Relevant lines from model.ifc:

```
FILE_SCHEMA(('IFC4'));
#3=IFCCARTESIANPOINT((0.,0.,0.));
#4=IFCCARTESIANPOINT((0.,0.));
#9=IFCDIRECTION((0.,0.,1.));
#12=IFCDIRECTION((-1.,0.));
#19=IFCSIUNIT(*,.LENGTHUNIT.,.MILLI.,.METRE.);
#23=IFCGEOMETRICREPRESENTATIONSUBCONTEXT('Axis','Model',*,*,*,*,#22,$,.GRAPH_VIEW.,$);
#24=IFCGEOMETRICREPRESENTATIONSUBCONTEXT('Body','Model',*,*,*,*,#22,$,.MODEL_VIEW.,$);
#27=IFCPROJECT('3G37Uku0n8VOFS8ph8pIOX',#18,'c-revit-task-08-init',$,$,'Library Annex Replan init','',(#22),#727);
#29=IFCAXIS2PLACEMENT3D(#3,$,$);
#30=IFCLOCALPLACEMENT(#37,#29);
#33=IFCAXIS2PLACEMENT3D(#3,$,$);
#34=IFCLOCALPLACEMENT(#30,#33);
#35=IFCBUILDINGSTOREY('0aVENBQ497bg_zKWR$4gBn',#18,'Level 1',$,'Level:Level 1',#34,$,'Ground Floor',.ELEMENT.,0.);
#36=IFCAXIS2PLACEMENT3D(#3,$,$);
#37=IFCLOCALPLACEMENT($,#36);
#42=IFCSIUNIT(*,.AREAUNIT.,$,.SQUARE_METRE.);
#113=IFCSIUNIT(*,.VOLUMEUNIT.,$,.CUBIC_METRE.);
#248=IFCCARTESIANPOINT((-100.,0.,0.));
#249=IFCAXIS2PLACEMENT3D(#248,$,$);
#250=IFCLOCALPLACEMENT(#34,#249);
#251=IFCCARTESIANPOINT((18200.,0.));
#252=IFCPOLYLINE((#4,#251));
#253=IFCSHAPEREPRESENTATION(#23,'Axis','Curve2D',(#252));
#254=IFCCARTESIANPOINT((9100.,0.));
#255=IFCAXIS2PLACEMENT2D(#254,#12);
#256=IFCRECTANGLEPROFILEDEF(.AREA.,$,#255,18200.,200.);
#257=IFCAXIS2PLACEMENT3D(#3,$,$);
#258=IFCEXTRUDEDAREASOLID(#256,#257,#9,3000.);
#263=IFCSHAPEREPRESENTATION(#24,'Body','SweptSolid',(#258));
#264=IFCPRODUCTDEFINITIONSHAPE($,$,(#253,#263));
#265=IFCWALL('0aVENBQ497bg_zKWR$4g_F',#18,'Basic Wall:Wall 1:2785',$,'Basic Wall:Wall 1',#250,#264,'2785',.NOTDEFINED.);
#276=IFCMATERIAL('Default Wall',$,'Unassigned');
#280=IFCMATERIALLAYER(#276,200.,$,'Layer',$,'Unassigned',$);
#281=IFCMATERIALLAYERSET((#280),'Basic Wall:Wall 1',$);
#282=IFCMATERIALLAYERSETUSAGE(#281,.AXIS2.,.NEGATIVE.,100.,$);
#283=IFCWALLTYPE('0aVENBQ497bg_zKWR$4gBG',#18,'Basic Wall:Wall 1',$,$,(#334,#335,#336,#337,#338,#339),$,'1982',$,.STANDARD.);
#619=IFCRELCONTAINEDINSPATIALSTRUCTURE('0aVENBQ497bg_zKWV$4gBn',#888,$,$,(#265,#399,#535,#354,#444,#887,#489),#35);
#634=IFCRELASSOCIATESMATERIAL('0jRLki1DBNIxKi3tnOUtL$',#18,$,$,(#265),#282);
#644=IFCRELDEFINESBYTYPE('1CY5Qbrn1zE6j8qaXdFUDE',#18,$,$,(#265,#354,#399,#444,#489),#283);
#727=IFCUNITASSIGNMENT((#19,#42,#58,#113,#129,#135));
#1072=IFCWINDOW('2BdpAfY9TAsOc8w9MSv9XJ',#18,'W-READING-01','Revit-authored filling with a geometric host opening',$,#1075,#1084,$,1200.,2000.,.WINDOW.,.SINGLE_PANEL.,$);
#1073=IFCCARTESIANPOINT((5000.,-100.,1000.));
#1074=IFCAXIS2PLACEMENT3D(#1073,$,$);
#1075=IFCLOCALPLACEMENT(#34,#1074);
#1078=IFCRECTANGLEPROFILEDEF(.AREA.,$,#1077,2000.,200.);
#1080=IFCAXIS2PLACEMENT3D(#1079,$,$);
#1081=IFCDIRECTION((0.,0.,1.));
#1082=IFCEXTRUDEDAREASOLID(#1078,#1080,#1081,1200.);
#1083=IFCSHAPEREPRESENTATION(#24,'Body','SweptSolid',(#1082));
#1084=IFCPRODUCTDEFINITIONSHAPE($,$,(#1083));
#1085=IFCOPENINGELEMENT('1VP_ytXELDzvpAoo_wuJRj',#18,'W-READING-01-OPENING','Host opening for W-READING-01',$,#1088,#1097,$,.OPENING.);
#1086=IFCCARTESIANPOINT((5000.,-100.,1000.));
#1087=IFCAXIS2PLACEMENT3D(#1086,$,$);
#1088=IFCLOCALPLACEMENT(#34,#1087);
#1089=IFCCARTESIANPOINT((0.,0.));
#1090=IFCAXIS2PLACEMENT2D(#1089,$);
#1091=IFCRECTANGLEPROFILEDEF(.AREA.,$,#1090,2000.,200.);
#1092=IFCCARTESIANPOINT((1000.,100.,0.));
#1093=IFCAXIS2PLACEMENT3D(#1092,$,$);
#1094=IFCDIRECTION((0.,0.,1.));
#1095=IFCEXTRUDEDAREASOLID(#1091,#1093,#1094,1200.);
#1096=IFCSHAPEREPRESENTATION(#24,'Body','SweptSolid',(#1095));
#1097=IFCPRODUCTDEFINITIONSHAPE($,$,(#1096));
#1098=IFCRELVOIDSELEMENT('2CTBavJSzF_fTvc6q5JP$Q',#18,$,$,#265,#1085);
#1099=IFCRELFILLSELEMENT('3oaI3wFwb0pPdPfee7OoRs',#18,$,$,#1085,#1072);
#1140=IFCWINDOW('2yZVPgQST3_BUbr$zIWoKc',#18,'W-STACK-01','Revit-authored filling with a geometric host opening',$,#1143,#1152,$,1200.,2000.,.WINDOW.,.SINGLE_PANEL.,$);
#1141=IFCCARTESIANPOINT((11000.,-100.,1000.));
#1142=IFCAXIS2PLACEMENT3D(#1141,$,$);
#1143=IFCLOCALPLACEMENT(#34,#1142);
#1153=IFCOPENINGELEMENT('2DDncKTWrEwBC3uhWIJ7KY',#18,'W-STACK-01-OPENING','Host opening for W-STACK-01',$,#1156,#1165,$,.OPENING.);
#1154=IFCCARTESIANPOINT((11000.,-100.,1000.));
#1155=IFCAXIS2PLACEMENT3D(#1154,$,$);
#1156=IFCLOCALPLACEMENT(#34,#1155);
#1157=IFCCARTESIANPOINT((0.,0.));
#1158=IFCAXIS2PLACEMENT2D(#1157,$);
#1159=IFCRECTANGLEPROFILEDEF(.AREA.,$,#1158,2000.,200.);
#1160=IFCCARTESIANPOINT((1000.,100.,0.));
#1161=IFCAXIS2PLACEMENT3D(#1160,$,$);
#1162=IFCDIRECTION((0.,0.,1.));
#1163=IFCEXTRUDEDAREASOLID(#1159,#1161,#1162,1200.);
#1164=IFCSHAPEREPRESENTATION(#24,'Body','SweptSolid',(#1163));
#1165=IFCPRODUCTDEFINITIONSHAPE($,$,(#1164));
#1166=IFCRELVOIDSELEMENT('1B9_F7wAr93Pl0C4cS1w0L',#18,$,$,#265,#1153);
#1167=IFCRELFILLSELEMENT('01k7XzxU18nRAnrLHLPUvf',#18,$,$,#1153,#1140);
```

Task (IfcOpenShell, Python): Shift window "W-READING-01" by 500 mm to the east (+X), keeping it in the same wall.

```python
import ifcopenshell
import ifcopenshell.api.geometry
import ifcopenshell.util.placement

model = ifcopenshell.open("model.ifc")

window = model.by_id(1072)
opening = window.FillsVoids[0].RelatingOpeningElement
wall = opening.VoidsElements[0].RelatingBuildingElement

wall_matrix = ifcopenshell.util.placement.get_local_placement(wall.ObjectPlacement)
shift = wall_matrix[:3, 0] * 500.0
before = ifcopenshell.util.placement.get_local_placement(window.ObjectPlacement)[:3, 3].copy()

# The window is not placed relative to its opening, so move both.
for product in (opening, window):
    matrix = ifcopenshell.util.placement.get_local_placement(product.ObjectPlacement)
    matrix[:3, 3] += shift
    ifcopenshell.api.geometry.edit_object_placement(model, product=product, matrix=matrix, is_si=False)

after = ifcopenshell.util.placement.get_local_placement(window.ObjectPlacement)[:3, 3]
print("window moved by", (after - before).round(3) + 0.0)

model.write("model_updated.ifc")
```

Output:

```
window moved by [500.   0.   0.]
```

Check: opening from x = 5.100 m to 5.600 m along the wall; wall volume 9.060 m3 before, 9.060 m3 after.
